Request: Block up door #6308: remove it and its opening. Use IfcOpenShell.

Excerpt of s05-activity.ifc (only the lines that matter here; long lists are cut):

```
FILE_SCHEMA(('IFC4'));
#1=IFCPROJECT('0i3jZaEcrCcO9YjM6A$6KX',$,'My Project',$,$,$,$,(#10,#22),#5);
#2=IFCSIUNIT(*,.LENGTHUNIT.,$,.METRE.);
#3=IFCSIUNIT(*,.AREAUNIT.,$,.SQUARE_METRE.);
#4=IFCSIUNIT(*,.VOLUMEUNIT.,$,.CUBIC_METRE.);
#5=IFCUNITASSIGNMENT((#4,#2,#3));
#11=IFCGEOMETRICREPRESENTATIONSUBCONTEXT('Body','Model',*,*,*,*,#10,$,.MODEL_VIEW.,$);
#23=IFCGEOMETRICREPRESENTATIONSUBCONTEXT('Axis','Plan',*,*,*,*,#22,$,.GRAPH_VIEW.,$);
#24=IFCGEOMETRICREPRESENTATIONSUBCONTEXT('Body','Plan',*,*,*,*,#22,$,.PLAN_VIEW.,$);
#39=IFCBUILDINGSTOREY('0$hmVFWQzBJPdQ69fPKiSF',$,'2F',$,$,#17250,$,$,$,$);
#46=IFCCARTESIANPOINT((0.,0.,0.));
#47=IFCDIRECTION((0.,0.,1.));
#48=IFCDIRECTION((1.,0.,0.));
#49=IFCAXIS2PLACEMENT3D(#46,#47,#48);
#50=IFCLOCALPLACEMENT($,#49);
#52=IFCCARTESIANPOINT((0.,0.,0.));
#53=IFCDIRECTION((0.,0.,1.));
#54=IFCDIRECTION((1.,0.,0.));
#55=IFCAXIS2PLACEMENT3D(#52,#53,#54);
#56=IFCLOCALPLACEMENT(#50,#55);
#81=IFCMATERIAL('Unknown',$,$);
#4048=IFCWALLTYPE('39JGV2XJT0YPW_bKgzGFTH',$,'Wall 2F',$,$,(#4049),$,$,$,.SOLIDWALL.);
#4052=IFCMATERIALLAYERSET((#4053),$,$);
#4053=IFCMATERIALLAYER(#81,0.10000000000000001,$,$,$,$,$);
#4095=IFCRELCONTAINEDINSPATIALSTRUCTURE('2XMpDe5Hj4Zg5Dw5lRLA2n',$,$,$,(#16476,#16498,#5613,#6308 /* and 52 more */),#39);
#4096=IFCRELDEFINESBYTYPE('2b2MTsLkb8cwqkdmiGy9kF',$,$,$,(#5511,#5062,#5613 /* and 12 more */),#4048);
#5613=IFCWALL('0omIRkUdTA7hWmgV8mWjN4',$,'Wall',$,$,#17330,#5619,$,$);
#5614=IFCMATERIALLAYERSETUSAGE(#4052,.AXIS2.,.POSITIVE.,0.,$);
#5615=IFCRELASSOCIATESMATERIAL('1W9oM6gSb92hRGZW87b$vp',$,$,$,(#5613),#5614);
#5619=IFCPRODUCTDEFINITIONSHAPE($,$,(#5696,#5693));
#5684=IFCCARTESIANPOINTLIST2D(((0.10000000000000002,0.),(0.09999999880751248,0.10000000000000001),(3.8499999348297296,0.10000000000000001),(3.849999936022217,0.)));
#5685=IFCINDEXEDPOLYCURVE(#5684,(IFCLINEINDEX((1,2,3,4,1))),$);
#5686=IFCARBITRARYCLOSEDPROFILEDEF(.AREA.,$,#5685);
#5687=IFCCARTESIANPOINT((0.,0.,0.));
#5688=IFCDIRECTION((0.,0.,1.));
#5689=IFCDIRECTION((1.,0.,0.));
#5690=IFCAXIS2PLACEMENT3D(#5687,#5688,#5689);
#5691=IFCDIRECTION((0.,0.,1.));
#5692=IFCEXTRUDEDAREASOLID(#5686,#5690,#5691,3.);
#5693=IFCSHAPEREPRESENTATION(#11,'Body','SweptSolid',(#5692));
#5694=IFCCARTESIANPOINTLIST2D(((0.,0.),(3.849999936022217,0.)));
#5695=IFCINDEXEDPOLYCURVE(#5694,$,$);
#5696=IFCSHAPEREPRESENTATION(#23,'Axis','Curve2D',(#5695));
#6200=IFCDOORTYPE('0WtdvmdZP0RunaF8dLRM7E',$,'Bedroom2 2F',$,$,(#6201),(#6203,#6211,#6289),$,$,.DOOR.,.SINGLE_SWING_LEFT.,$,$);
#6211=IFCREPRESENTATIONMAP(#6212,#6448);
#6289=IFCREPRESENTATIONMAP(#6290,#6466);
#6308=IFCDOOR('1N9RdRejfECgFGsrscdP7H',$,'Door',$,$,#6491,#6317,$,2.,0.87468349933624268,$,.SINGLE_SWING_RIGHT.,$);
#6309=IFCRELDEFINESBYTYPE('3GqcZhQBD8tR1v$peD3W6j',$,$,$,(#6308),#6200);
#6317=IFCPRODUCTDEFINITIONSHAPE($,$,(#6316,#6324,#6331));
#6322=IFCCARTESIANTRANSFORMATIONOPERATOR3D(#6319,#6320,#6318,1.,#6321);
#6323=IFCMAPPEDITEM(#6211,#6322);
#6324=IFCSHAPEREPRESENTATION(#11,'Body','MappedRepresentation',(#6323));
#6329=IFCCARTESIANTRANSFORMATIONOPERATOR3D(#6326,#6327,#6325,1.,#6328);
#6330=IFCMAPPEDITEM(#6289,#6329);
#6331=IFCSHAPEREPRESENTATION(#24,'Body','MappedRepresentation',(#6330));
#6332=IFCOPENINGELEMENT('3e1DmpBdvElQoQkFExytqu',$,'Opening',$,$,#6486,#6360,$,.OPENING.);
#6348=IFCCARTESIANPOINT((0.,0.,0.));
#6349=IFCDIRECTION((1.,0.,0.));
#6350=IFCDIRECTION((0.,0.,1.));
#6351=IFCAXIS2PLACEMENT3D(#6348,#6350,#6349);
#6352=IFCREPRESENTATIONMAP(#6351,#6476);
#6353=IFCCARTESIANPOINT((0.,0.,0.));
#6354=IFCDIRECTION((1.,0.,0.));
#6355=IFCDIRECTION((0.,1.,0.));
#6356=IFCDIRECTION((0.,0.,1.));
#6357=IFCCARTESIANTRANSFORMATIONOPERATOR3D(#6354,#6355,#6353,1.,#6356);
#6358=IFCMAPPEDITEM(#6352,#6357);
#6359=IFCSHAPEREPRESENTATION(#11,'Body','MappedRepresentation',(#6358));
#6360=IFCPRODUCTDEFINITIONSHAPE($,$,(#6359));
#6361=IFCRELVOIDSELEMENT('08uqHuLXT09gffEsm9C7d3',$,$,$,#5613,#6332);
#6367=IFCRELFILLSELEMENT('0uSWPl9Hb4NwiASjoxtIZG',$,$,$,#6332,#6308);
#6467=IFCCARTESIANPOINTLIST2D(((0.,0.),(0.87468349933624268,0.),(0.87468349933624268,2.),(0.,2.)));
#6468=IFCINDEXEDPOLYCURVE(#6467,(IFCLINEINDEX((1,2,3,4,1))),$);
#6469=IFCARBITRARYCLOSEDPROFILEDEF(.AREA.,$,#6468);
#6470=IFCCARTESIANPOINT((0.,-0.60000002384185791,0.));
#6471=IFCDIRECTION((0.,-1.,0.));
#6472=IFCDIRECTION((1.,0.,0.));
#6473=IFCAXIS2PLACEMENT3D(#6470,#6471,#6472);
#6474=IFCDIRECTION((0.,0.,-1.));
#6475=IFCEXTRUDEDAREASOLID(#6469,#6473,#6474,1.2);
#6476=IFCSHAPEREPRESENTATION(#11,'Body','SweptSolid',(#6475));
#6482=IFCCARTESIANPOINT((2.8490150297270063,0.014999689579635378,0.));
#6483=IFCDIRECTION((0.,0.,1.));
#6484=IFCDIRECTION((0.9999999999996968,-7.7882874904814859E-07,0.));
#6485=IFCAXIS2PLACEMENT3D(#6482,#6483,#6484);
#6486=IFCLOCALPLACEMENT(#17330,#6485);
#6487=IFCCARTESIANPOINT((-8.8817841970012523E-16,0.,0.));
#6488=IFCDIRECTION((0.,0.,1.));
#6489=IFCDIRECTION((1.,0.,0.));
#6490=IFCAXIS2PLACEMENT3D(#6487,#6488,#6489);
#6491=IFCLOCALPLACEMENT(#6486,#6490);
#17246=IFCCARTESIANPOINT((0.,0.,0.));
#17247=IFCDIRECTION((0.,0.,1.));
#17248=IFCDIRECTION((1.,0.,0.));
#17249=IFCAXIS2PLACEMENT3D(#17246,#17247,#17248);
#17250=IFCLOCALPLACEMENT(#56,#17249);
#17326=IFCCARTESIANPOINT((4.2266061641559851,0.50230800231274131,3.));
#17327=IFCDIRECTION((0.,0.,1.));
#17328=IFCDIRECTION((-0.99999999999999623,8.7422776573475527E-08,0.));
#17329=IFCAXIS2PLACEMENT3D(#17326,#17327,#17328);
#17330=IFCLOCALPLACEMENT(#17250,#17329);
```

```python
import ifcopenshell
import ifcopenshell.api.feature
import ifcopenshell.api.root
import ifcopenshell.geom
import ifcopenshell.util.shape

model = ifcopenshell.open("s05-activity.ifc")
settings = ifcopenshell.geom.settings()


def volume(element):
    """Net volume in cubic metres, openings subtracted."""
    shape = ifcopenshell.geom.create_shape(settings, element)
    return ifcopenshell.util.shape.get_volume(shape.geometry)


door = model.by_guid("1N9RdRejfECgFGsrscdP7H")
opening = door.FillsVoids[0].RelatingOpeningElement
wall = opening.VoidsElements[0].RelatingBuildingElement
before = volume(wall)

ifcopenshell.api.root.remove_product(model, product=door)
ifcopenshell.api.feature.remove_feature(model, feature=opening)

after = volume(wall)

print(f"wall volume {before:.3f} -> {after:.3f} m3")

model.write("s05-activity_v2.ifc")
```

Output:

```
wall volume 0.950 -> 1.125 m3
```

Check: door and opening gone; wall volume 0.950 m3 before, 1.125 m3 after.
